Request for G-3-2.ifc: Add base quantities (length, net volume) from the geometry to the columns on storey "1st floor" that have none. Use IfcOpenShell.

First a look at what the model holds.

```python
import ifcopenshell
import ifcopenshell.util.element
import ifcopenshell.util.unit

model = ifcopenshell.open("G-3-2.ifc")
print(model.schema)
for unit_type in ("LENGTHUNIT", "AREAUNIT", "VOLUMEUNIT"):
    print(unit_type, ifcopenshell.util.unit.calculate_unit_scale(model, unit_type))
storey = next(s for s in model.by_type("IfcBuildingStorey") if s.Name == "1st floor")
columns = [e for e in ifcopenshell.util.element.get_decomposition(storey) if e.is_a("IfcColumn")]
for e in sorted(columns, key=lambda e: e.id()):
    print(e.id(), e.is_a(), e.Name, list(ifcopenshell.util.element.get_psets(e, qtos_only=True)), sep=" | ")
```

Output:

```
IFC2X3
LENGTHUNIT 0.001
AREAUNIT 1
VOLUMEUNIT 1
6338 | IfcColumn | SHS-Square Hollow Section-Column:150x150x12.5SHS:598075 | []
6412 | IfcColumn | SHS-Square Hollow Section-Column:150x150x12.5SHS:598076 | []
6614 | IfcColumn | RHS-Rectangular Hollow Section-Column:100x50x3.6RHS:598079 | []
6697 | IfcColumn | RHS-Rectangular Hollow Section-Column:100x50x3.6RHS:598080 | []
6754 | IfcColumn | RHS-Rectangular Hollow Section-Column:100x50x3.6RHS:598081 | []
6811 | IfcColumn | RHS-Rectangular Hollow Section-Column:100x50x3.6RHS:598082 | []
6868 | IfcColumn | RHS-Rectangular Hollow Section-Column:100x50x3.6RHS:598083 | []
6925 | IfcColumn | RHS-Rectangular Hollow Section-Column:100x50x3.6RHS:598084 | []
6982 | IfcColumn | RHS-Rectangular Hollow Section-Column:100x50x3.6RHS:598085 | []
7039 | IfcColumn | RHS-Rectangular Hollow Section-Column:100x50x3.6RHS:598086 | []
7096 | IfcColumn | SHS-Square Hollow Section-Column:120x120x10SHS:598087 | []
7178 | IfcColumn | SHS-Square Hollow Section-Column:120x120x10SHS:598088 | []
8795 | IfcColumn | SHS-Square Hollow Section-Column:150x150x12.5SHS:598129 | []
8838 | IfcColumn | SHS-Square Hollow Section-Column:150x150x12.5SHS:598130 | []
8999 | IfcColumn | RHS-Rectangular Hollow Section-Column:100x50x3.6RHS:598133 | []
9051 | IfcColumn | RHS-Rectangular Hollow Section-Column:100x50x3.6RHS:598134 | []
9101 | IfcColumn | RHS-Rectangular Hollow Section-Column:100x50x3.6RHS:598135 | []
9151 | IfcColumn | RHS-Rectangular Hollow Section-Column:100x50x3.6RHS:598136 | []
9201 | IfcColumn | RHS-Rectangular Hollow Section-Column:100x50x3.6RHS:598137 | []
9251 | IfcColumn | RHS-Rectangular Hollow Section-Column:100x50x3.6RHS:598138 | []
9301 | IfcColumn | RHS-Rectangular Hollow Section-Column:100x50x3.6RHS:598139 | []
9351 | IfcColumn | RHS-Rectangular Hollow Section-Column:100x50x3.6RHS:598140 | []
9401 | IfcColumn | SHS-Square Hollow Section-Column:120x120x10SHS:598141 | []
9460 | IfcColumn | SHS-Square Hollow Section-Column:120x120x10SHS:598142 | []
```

```python
import ifcopenshell
import ifcopenshell.api.pset
import ifcopenshell.geom
import ifcopenshell.util.element
import ifcopenshell.util.shape
import ifcopenshell.util.unit

model = ifcopenshell.open("G-3-2.ifc")
unit_scale = ifcopenshell.util.unit.calculate_unit_scale(model)
volume_scale = ifcopenshell.util.unit.calculate_unit_scale(model, "VOLUMEUNIT")
settings = ifcopenshell.geom.settings()

storey = next(s for s in model.by_type("IfcBuildingStorey") if s.Name == "1st floor")
columns = [e for e in ifcopenshell.util.element.get_decomposition(storey) if e.is_a("IfcColumn")]

for e in sorted(columns, key=lambda e: e.id()):
    if ifcopenshell.util.element.get_psets(e, qtos_only=True, should_inherit=False):
        continue
    # Geometry comes back in metres, in the element's own axes.
    shape = ifcopenshell.geom.create_shape(settings, e)
    values = {
        "Length": ifcopenshell.util.shape.get_z(shape.geometry) / unit_scale,
        "NetVolume": ifcopenshell.util.shape.get_volume(shape.geometry) / volume_scale,
    }
    qto = ifcopenshell.api.pset.add_qto(model, product=e, name="BaseQuantities")
    ifcopenshell.api.pset.edit_qto(model, qto=qto, properties=values)
    print(e.id(), {k: round(v, 3) for k, v in values.items()})

model.write("G-3-2_v2.ifc")
```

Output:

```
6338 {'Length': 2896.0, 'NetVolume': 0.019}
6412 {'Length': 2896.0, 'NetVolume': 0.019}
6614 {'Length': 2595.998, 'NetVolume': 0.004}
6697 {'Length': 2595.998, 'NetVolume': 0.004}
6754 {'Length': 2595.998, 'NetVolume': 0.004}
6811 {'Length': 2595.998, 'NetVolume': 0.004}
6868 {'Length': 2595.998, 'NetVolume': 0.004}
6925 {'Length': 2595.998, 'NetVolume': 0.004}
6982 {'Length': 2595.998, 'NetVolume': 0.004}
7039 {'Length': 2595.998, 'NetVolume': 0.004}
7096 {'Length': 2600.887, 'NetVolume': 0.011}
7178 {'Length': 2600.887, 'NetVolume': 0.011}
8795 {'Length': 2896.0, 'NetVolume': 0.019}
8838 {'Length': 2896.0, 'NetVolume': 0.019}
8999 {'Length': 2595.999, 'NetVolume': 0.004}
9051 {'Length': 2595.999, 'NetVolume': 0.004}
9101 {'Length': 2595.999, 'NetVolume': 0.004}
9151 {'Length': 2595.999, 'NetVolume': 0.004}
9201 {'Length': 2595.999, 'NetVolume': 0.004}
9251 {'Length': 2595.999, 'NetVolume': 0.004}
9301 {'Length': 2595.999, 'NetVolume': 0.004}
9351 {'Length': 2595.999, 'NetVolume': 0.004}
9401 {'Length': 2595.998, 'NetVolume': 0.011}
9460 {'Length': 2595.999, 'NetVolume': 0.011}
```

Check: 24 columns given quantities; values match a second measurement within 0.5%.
